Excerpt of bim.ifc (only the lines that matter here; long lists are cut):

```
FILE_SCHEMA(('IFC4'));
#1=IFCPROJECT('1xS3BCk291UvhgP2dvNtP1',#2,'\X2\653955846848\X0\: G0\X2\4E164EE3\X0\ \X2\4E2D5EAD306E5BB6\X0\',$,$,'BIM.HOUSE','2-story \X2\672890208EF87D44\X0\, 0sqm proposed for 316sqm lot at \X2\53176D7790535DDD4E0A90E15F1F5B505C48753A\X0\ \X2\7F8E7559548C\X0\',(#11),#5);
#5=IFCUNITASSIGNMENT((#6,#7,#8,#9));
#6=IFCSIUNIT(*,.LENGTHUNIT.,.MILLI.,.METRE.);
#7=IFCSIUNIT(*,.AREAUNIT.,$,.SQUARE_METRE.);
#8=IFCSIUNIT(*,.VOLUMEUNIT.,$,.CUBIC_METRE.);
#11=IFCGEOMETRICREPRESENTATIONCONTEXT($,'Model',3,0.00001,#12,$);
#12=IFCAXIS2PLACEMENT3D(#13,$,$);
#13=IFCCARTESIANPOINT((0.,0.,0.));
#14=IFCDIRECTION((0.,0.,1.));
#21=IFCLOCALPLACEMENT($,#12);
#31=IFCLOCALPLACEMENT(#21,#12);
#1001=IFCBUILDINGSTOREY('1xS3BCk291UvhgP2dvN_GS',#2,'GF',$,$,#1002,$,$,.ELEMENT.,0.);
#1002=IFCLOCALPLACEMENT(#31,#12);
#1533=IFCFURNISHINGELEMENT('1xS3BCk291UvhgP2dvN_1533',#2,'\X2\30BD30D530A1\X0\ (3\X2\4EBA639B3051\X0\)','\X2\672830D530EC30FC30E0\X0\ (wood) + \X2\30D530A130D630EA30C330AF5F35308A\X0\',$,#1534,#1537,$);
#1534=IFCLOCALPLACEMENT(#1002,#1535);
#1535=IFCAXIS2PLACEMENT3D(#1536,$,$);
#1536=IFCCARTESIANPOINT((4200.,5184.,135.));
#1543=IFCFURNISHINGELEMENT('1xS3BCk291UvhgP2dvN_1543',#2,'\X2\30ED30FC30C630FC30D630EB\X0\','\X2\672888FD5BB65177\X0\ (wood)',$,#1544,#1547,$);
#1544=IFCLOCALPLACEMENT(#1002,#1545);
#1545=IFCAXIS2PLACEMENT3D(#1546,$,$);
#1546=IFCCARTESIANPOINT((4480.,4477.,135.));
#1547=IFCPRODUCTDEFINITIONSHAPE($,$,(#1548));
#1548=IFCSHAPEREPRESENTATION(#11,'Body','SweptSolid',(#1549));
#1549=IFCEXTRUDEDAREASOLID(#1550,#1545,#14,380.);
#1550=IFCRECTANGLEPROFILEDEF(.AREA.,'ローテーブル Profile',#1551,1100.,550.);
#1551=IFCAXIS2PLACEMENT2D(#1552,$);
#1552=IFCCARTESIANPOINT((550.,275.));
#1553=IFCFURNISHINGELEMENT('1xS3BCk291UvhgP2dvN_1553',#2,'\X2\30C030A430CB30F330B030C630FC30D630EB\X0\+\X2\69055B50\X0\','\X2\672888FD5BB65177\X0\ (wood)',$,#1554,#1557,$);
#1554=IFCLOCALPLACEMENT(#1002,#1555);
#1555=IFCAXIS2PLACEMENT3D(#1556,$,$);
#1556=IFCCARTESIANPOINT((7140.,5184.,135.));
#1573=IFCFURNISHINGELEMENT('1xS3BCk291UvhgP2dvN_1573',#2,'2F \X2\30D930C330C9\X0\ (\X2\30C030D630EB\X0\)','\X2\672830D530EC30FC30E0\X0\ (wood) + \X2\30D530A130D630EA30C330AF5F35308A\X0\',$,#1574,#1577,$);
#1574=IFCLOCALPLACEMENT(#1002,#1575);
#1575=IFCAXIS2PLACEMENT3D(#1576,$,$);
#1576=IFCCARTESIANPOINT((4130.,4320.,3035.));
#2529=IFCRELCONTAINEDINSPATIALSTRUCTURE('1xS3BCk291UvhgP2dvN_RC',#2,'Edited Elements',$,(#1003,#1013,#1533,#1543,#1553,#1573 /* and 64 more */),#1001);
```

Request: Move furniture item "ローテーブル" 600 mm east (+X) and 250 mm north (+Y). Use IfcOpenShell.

```python
import ifcopenshell
import ifcopenshell.api.geometry
import ifcopenshell.util.placement

model = ifcopenshell.open("bim.ifc")

item = model.by_guid("1xS3BCk291UvhgP2dvN_1543")
matrix = ifcopenshell.util.placement.get_local_placement(item.ObjectPlacement)
matrix[0, 3] += 600.0
matrix[1, 3] += 250.0
ifcopenshell.api.geometry.edit_object_placement(model, product=item, matrix=matrix, is_si=False)

print(ifcopenshell.util.placement.get_local_placement(item.ObjectPlacement).round(3) + 0.0)

model.write("bim_rev.ifc")
```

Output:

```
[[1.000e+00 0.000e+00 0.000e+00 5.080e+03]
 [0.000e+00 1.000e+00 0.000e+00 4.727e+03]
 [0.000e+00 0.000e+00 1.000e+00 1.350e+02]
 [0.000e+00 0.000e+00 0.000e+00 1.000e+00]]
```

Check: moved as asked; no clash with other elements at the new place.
